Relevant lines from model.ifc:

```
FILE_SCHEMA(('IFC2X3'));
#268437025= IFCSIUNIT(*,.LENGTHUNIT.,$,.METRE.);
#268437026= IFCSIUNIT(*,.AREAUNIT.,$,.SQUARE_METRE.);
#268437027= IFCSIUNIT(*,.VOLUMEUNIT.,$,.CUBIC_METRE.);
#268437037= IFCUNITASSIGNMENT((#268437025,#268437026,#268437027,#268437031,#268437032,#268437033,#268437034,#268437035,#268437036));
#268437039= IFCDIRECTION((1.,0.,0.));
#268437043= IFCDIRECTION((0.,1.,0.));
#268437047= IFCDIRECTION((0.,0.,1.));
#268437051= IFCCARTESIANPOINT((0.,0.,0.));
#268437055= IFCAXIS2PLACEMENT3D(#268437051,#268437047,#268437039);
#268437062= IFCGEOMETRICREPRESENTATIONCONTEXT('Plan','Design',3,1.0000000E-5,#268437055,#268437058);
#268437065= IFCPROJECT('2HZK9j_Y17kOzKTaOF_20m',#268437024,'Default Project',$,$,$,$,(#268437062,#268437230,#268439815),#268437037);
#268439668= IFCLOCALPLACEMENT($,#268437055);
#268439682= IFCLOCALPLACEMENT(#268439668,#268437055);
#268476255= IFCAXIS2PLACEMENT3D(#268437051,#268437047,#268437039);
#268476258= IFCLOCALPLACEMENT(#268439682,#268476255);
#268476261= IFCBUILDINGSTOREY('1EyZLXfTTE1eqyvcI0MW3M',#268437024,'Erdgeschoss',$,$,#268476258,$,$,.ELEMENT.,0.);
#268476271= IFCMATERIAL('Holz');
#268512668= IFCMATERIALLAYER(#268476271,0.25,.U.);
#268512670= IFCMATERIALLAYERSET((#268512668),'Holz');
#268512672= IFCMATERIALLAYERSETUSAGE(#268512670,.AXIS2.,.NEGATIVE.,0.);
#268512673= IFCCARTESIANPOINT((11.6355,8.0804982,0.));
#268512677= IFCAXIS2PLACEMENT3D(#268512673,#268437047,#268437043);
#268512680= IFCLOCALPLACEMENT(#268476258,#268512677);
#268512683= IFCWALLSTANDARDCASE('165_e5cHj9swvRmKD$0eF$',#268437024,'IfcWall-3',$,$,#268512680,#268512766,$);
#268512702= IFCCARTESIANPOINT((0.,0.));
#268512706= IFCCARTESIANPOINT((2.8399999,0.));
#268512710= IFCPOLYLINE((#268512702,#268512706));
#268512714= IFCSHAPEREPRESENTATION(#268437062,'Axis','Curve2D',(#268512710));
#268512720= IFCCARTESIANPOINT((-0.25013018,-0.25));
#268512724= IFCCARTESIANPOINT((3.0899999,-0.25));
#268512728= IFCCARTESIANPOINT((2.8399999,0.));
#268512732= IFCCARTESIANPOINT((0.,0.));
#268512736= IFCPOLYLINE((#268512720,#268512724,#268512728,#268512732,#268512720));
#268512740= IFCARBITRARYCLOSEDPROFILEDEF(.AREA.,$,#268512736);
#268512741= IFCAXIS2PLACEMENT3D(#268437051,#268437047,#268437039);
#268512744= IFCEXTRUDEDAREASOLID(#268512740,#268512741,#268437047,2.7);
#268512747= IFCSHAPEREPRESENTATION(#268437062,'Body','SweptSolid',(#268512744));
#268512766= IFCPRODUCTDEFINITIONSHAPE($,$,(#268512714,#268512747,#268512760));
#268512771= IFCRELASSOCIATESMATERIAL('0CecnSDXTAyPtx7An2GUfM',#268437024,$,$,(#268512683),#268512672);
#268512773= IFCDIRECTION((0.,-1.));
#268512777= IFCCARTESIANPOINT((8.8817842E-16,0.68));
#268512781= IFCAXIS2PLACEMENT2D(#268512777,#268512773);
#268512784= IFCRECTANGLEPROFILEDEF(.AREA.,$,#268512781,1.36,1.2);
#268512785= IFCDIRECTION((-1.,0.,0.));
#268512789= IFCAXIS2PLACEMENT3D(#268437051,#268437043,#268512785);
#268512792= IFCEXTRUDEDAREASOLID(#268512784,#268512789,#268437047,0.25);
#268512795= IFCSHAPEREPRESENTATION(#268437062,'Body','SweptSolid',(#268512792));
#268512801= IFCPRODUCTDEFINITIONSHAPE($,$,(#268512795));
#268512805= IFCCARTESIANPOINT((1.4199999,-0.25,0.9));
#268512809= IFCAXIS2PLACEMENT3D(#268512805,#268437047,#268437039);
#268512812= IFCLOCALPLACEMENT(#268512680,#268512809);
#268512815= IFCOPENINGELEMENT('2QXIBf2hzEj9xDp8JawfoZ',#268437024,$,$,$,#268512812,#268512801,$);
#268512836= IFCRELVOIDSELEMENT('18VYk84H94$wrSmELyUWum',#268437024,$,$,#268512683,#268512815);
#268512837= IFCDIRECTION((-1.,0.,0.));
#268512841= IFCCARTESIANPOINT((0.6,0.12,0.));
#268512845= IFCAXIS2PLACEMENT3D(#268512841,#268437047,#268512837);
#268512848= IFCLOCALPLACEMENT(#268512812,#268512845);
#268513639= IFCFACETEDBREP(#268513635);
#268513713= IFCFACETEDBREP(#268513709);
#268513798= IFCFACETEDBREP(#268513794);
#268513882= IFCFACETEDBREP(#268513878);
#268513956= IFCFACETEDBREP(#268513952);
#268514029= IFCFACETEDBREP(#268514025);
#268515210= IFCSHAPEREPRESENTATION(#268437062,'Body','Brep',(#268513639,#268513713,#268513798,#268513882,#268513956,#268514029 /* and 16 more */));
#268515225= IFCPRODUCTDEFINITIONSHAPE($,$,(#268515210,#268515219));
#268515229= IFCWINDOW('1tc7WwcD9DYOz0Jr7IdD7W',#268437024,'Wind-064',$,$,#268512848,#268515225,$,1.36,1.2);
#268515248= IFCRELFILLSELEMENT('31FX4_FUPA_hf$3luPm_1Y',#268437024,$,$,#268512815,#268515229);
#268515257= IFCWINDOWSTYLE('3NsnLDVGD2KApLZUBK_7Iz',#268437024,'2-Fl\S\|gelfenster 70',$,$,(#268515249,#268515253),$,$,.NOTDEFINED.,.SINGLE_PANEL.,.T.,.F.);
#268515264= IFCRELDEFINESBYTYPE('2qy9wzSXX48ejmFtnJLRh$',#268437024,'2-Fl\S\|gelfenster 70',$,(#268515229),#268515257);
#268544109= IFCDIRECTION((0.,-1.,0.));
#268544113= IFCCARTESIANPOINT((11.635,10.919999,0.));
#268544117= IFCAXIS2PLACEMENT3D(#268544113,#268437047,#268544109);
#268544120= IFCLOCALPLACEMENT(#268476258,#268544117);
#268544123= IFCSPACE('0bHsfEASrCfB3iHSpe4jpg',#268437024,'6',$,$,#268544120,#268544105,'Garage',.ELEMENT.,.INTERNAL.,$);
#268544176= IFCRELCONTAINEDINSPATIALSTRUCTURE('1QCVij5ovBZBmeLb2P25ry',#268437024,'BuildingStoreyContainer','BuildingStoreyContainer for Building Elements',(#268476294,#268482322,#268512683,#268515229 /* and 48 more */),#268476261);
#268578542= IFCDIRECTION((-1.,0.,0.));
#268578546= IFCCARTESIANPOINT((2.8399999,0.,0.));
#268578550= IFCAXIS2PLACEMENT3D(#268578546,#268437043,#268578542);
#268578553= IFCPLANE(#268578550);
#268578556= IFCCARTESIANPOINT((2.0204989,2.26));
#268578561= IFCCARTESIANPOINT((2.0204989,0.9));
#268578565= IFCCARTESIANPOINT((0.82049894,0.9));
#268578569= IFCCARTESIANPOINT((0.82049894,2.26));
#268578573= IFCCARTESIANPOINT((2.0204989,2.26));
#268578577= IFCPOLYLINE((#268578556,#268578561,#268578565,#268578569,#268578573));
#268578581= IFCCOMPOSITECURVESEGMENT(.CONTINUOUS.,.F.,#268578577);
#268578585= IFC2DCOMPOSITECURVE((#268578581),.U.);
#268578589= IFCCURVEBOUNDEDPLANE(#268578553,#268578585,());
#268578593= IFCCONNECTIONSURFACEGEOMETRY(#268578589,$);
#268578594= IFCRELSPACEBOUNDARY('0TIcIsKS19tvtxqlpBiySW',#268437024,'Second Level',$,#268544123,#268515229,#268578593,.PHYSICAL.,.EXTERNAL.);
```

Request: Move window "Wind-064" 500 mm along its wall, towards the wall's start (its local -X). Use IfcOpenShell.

```python
import numpy as np
import ifcopenshell
import ifcopenshell.api.geometry
import ifcopenshell.util.placement
import ifcopenshell.util.unit

model = ifcopenshell.open("model.ifc")
unit_scale = ifcopenshell.util.unit.calculate_unit_scale(model)

window = model.by_guid("1tc7WwcD9DYOz0Jr7IdD7W")
opening = window.FillsVoids[0].RelatingOpeningElement
wall = opening.VoidsElements[0].RelatingBuildingElement

wall_matrix = ifcopenshell.util.placement.get_local_placement(wall.ObjectPlacement)
shift = wall_matrix[:3, 0] * -0.5 / unit_scale
before = ifcopenshell.util.placement.get_local_placement(window.ObjectPlacement)[:3, 3].copy()

# The window is placed relative to its opening, so it follows when the opening moves.
matrix = ifcopenshell.util.placement.get_local_placement(opening.ObjectPlacement)
matrix[:3, 3] += shift
ifcopenshell.api.geometry.edit_object_placement(
    model, product=opening, matrix=matrix, is_si=False, should_transform_children=True
)

# Space boundary surfaces are stored in each space's coordinates; move them too.
for rel in window.ProvidesBoundaries:
    if not rel.ConnectionGeometry:
        continue
    surface = rel.ConnectionGeometry.SurfaceOnRelatingElement.BasisSurface
    space_matrix = ifcopenshell.util.placement.get_local_placement(rel.RelatingSpace.ObjectPlacement)
    point = np.array(surface.Position.Location.Coordinates) + space_matrix[:3, :3].T @ shift
    surface.Position = model.createIfcAxis2Placement3D(
        model.createIfcCartesianPoint(point.tolist()), surface.Position.Axis, surface.Position.RefDirection
    )

after = ifcopenshell.util.placement.get_local_placement(window.ObjectPlacement)[:3, 3]
print("window moved by", (after - before).round(3) + 0.0)

model.write("model-out.ifc")
```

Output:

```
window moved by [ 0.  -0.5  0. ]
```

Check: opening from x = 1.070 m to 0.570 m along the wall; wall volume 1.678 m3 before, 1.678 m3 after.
